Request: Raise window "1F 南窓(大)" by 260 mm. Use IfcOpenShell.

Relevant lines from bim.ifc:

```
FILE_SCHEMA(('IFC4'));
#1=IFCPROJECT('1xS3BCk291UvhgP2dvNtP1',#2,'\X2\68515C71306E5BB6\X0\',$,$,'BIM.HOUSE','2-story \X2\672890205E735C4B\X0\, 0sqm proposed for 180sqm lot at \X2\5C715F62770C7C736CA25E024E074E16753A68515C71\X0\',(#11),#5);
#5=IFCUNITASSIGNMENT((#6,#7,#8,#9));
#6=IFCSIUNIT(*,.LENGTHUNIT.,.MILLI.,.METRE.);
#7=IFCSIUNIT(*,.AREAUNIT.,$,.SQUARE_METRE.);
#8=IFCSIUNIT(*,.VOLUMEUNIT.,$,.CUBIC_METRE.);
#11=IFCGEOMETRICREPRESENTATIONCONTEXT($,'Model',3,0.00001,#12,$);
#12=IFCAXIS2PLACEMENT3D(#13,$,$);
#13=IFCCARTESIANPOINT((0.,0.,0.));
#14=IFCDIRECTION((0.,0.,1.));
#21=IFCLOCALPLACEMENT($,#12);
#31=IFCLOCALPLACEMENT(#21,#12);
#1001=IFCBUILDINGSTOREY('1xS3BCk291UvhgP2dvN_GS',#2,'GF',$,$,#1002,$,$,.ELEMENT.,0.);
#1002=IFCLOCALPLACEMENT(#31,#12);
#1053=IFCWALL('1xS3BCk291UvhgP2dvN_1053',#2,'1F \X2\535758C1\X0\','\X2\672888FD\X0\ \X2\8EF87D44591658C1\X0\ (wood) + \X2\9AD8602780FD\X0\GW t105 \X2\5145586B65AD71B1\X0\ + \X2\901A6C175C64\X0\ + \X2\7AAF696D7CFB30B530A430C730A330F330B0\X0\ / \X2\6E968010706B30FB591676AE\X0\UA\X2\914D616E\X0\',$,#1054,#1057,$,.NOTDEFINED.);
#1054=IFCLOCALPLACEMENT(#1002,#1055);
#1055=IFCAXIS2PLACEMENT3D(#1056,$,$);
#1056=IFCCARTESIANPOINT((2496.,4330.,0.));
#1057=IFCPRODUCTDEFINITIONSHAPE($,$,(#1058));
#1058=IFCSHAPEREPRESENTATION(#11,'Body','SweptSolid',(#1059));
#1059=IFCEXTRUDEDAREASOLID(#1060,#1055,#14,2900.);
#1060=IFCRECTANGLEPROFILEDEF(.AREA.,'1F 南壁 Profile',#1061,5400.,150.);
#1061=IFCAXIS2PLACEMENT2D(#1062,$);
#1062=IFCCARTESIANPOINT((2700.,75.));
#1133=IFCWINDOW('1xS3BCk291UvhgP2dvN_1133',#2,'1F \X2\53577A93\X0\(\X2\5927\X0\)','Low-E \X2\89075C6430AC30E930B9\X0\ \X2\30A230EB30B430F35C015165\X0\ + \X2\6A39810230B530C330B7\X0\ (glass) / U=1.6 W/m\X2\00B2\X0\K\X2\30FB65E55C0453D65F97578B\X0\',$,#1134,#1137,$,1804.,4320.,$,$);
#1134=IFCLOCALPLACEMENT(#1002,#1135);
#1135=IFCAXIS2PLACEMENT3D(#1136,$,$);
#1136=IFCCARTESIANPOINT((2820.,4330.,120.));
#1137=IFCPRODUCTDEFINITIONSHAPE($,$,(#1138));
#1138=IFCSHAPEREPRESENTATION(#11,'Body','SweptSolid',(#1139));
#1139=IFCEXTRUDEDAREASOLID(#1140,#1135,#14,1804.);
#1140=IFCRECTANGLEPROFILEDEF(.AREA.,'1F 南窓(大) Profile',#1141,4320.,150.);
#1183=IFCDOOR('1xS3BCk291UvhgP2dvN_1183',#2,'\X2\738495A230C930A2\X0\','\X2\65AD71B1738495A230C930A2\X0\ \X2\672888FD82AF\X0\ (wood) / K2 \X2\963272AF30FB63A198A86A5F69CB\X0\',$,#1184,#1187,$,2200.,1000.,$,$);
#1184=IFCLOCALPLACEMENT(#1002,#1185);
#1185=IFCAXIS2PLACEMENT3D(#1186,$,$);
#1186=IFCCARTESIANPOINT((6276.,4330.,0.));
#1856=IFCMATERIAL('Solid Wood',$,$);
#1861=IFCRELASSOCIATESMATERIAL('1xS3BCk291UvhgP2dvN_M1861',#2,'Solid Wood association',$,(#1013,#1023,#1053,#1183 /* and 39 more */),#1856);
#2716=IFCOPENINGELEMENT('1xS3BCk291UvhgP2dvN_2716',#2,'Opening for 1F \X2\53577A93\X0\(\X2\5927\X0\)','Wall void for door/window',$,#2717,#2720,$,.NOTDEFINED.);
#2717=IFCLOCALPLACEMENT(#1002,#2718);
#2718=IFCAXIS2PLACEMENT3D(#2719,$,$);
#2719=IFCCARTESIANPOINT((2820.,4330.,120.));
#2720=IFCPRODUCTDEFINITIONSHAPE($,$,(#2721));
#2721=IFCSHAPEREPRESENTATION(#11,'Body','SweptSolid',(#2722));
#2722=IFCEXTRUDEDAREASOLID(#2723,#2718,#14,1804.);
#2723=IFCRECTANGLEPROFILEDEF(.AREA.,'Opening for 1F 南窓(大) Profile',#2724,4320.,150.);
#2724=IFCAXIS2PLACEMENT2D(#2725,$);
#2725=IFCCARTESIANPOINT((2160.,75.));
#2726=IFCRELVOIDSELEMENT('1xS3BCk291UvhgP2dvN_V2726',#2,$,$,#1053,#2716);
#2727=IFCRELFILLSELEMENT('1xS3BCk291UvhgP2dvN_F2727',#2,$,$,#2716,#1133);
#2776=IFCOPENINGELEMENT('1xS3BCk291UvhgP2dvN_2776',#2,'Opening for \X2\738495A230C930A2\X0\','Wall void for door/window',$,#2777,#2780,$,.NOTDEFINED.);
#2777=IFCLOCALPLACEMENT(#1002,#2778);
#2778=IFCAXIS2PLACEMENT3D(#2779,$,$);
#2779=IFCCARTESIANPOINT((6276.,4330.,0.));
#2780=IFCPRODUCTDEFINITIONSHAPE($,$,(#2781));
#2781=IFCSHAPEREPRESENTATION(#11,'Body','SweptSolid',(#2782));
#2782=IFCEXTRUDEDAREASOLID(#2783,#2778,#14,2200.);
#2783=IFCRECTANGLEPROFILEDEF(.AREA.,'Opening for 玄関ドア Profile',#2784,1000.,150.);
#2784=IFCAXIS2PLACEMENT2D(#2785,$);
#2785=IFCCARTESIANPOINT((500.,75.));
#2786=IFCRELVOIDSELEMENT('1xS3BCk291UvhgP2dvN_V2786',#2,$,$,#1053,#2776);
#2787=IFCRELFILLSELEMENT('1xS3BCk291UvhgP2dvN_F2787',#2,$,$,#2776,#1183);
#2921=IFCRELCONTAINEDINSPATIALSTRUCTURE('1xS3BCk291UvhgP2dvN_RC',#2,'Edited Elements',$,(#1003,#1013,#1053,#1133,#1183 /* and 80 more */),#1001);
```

```python
import numpy as np
import ifcopenshell
import ifcopenshell.api.geometry
import ifcopenshell.util.placement
import ifcopenshell.util.unit

model = ifcopenshell.open("bim.ifc")
unit_scale = ifcopenshell.util.unit.calculate_unit_scale(model)

window = model.by_guid("1xS3BCk291UvhgP2dvN_1133")
opening = window.FillsVoids[0].RelatingOpeningElement
dz = 0.26 / unit_scale

shift = np.array([0.0, 0.0, dz])
# The window is not placed relative to its opening, so move both.
for product in (opening, window):
    matrix = ifcopenshell.util.placement.get_local_placement(product.ObjectPlacement)
    matrix[:3, 3] += shift
    ifcopenshell.api.geometry.edit_object_placement(model, product=product, matrix=matrix, is_si=False)

print(f"moved by {dz * unit_scale:+.3f} m")

model.write("bim_v2.ifc")
```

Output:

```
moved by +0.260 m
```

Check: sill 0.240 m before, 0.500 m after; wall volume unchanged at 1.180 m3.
